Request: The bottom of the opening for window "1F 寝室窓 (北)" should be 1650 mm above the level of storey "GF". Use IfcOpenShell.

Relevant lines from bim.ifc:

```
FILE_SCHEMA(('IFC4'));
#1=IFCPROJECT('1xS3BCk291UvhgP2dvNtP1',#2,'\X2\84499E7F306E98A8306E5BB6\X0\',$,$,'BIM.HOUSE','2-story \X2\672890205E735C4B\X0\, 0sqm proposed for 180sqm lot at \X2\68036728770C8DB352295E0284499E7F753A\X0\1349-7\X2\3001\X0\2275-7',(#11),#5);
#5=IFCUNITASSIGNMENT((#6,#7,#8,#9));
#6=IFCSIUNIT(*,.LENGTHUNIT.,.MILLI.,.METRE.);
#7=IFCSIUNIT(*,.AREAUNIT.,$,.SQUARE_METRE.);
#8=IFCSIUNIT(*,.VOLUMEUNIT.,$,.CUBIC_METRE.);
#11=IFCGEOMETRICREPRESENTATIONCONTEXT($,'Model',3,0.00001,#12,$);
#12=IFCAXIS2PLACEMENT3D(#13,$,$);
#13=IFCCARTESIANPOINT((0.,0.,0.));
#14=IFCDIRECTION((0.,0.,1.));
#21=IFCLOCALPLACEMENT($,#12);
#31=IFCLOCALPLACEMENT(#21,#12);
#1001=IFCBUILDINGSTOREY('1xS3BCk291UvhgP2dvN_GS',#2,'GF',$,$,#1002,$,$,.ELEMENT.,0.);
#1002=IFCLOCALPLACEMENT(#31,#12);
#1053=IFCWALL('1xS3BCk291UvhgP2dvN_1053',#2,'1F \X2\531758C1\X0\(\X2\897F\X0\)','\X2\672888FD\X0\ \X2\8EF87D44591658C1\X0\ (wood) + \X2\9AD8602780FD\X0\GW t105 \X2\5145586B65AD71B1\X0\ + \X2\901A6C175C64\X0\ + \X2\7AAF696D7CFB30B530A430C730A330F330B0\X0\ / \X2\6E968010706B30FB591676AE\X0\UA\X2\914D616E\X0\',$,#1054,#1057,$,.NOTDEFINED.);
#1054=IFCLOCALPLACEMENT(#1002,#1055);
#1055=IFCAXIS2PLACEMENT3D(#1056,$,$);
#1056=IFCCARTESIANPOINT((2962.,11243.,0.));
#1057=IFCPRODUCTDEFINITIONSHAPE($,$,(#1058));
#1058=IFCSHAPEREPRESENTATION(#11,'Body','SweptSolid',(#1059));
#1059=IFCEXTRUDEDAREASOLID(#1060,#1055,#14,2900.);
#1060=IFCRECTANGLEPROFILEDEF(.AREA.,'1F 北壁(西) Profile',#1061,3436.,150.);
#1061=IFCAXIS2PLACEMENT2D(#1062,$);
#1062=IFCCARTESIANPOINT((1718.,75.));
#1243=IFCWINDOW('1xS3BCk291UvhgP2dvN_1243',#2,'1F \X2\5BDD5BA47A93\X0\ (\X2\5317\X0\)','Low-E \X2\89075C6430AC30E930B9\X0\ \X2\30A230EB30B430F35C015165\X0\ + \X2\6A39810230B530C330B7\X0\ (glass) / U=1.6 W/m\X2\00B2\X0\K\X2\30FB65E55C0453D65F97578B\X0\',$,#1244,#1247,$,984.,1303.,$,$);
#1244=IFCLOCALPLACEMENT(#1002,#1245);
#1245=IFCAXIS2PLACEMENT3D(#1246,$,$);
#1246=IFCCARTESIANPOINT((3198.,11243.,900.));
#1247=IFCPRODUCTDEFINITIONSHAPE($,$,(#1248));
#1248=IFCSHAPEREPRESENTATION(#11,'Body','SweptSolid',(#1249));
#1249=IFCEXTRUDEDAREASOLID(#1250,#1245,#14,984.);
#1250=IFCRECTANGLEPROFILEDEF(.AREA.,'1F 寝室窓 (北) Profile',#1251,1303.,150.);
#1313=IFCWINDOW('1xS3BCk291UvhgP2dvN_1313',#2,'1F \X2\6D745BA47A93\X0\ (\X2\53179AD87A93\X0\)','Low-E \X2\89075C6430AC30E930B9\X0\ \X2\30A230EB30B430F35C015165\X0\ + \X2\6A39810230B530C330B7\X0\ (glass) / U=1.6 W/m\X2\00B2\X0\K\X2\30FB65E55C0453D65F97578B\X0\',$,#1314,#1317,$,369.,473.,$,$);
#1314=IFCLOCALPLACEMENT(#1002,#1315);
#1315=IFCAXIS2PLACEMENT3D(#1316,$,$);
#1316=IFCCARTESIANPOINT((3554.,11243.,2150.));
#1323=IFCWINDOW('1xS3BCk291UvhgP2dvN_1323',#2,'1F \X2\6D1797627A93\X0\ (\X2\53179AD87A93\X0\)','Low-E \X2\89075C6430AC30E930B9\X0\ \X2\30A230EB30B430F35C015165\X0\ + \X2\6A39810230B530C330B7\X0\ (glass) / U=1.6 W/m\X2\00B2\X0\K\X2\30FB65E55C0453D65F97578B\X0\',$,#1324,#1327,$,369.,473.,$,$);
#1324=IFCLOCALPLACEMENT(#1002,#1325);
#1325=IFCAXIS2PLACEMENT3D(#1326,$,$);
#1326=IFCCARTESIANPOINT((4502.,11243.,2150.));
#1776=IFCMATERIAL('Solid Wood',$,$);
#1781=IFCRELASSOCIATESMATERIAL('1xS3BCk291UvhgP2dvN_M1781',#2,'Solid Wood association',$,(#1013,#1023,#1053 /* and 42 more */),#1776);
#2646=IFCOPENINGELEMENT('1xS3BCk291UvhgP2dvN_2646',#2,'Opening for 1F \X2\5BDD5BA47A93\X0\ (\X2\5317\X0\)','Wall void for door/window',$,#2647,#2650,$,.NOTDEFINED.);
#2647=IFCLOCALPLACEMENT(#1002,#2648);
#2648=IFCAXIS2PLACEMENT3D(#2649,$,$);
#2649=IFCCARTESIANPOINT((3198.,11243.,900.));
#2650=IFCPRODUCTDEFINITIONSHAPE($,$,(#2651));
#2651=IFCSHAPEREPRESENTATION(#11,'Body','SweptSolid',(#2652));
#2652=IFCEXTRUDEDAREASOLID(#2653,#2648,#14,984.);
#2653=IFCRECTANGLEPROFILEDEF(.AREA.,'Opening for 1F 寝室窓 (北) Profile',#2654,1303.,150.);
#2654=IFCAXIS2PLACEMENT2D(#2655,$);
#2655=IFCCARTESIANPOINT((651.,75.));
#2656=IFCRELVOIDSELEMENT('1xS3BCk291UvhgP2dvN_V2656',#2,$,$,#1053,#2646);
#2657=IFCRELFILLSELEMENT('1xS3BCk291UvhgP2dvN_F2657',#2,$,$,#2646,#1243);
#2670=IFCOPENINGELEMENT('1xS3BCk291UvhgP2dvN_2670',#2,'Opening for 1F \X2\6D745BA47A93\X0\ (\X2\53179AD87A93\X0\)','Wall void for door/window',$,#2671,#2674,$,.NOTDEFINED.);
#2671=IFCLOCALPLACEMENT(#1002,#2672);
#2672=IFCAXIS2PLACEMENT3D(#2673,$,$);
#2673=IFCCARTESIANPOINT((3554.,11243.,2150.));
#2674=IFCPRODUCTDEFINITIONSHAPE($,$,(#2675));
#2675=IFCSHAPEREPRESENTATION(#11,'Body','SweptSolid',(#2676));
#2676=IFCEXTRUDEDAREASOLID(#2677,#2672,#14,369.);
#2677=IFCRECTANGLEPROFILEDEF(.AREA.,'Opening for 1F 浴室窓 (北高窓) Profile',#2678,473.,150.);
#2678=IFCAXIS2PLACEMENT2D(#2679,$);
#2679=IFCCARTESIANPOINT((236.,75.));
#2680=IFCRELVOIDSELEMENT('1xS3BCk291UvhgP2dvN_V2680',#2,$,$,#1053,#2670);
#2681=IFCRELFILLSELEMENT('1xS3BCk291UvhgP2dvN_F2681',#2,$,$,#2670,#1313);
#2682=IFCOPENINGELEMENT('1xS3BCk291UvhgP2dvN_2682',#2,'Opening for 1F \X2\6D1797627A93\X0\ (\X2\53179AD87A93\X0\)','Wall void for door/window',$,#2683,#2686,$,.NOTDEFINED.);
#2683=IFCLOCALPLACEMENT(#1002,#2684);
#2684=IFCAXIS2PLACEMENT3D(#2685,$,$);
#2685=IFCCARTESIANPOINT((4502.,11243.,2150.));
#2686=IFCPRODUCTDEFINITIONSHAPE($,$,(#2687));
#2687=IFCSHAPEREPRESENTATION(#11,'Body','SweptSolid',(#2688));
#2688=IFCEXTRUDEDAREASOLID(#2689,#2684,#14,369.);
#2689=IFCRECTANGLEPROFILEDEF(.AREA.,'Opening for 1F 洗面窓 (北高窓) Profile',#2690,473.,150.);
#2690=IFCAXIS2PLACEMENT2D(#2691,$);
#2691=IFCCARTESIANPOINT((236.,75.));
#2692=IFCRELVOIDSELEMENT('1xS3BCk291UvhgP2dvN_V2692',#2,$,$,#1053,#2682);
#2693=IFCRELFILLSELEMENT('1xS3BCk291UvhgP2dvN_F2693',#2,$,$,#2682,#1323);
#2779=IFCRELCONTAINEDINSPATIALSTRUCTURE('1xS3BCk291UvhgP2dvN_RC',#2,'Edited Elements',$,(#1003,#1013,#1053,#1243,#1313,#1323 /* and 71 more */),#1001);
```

```python
import numpy as np
import ifcopenshell
import ifcopenshell.api.geometry
import ifcopenshell.geom
import ifcopenshell.util.element
import ifcopenshell.util.placement
import ifcopenshell.util.shape
import ifcopenshell.util.unit

model = ifcopenshell.open("bim.ifc")
unit_scale = ifcopenshell.util.unit.calculate_unit_scale(model)

window = model.by_id(1243)
opening = window.FillsVoids[0].RelatingOpeningElement
storey = ifcopenshell.util.element.get_container(window, ifc_class="IfcBuildingStorey")
level = ifcopenshell.util.placement.get_local_placement(storey.ObjectPlacement)[2, 3]

# The opening's origin need not be at the sill, so measure its lowest point.
shape = ifcopenshell.geom.create_shape(ifcopenshell.geom.settings(), opening)
bottom = ifcopenshell.util.shape.get_shape_bottom_elevation(shape, shape.geometry) / unit_scale
dz = level + 1.65 / unit_scale - bottom

shift = np.array([0.0, 0.0, dz])
# The window is not placed relative to its opening, so move both.
for product in (opening, window):
    matrix = ifcopenshell.util.placement.get_local_placement(product.ObjectPlacement)
    matrix[:3, 3] += shift
    ifcopenshell.api.geometry.edit_object_placement(model, product=product, matrix=matrix, is_si=False)

print(f"moved by {dz * unit_scale:+.3f} m")

model.write("bim_edited.ifc")
```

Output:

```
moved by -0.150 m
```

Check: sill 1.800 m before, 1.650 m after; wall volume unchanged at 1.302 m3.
